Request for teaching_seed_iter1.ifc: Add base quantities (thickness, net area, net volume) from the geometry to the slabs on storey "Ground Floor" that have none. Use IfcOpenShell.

First a look at what the model holds.

```python
import ifcopenshell
import ifcopenshell.util.element
import ifcopenshell.util.unit

model = ifcopenshell.open("teaching_seed_iter1.ifc")
print(model.schema)
for unit_type in ("LENGTHUNIT", "AREAUNIT", "VOLUMEUNIT"):
    print(unit_type, ifcopenshell.util.unit.calculate_unit_scale(model, unit_type))
storey = next(s for s in model.by_type("IfcBuildingStorey") if s.Name == "Ground Floor")
slabs = [e for e in ifcopenshell.util.element.get_decomposition(storey) if e.is_a("IfcSlab")]
for e in sorted(slabs, key=lambda e: e.id()):
    print(e.id(), e.is_a(), e.Name, list(ifcopenshell.util.element.get_psets(e, qtos_only=True)), sep=" | ")
```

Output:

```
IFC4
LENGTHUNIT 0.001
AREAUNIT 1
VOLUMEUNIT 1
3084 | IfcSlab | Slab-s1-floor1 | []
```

```python
import ifcopenshell
import ifcopenshell.api.pset
import ifcopenshell.geom
import ifcopenshell.util.element
import ifcopenshell.util.shape
import ifcopenshell.util.unit

model = ifcopenshell.open("teaching_seed_iter1.ifc")
unit_scale = ifcopenshell.util.unit.calculate_unit_scale(model)
area_scale = ifcopenshell.util.unit.calculate_unit_scale(model, "AREAUNIT")
volume_scale = ifcopenshell.util.unit.calculate_unit_scale(model, "VOLUMEUNIT")
settings = ifcopenshell.geom.settings()

storey = next(s for s in model.by_type("IfcBuildingStorey") if s.Name == "Ground Floor")
slabs = [e for e in ifcopenshell.util.element.get_decomposition(storey) if e.is_a("IfcSlab")]

for e in sorted(slabs, key=lambda e: e.id()):
    if ifcopenshell.util.element.get_psets(e, qtos_only=True, should_inherit=False):
        continue
    # Geometry comes back in metres, in the element's own axes.
    shape = ifcopenshell.geom.create_shape(settings, e)
    values = {
        "Width": ifcopenshell.util.shape.get_z(shape.geometry) / unit_scale,
        "NetArea": ifcopenshell.util.shape.get_footprint_area(shape.geometry) / area_scale,
        "NetVolume": ifcopenshell.util.shape.get_volume(shape.geometry) / volume_scale,
    }
    qto = ifcopenshell.api.pset.add_qto(model, product=e, name="Qto_SlabBaseQuantities")
    ifcopenshell.api.pset.edit_qto(model, qto=qto, properties=values)
    print(e.id(), {k: round(v, 3) for k, v in values.items()})

model.write("teaching_seed_iter1_v2.ifc")
```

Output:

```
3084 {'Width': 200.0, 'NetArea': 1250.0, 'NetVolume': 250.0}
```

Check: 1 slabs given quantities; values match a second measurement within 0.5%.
